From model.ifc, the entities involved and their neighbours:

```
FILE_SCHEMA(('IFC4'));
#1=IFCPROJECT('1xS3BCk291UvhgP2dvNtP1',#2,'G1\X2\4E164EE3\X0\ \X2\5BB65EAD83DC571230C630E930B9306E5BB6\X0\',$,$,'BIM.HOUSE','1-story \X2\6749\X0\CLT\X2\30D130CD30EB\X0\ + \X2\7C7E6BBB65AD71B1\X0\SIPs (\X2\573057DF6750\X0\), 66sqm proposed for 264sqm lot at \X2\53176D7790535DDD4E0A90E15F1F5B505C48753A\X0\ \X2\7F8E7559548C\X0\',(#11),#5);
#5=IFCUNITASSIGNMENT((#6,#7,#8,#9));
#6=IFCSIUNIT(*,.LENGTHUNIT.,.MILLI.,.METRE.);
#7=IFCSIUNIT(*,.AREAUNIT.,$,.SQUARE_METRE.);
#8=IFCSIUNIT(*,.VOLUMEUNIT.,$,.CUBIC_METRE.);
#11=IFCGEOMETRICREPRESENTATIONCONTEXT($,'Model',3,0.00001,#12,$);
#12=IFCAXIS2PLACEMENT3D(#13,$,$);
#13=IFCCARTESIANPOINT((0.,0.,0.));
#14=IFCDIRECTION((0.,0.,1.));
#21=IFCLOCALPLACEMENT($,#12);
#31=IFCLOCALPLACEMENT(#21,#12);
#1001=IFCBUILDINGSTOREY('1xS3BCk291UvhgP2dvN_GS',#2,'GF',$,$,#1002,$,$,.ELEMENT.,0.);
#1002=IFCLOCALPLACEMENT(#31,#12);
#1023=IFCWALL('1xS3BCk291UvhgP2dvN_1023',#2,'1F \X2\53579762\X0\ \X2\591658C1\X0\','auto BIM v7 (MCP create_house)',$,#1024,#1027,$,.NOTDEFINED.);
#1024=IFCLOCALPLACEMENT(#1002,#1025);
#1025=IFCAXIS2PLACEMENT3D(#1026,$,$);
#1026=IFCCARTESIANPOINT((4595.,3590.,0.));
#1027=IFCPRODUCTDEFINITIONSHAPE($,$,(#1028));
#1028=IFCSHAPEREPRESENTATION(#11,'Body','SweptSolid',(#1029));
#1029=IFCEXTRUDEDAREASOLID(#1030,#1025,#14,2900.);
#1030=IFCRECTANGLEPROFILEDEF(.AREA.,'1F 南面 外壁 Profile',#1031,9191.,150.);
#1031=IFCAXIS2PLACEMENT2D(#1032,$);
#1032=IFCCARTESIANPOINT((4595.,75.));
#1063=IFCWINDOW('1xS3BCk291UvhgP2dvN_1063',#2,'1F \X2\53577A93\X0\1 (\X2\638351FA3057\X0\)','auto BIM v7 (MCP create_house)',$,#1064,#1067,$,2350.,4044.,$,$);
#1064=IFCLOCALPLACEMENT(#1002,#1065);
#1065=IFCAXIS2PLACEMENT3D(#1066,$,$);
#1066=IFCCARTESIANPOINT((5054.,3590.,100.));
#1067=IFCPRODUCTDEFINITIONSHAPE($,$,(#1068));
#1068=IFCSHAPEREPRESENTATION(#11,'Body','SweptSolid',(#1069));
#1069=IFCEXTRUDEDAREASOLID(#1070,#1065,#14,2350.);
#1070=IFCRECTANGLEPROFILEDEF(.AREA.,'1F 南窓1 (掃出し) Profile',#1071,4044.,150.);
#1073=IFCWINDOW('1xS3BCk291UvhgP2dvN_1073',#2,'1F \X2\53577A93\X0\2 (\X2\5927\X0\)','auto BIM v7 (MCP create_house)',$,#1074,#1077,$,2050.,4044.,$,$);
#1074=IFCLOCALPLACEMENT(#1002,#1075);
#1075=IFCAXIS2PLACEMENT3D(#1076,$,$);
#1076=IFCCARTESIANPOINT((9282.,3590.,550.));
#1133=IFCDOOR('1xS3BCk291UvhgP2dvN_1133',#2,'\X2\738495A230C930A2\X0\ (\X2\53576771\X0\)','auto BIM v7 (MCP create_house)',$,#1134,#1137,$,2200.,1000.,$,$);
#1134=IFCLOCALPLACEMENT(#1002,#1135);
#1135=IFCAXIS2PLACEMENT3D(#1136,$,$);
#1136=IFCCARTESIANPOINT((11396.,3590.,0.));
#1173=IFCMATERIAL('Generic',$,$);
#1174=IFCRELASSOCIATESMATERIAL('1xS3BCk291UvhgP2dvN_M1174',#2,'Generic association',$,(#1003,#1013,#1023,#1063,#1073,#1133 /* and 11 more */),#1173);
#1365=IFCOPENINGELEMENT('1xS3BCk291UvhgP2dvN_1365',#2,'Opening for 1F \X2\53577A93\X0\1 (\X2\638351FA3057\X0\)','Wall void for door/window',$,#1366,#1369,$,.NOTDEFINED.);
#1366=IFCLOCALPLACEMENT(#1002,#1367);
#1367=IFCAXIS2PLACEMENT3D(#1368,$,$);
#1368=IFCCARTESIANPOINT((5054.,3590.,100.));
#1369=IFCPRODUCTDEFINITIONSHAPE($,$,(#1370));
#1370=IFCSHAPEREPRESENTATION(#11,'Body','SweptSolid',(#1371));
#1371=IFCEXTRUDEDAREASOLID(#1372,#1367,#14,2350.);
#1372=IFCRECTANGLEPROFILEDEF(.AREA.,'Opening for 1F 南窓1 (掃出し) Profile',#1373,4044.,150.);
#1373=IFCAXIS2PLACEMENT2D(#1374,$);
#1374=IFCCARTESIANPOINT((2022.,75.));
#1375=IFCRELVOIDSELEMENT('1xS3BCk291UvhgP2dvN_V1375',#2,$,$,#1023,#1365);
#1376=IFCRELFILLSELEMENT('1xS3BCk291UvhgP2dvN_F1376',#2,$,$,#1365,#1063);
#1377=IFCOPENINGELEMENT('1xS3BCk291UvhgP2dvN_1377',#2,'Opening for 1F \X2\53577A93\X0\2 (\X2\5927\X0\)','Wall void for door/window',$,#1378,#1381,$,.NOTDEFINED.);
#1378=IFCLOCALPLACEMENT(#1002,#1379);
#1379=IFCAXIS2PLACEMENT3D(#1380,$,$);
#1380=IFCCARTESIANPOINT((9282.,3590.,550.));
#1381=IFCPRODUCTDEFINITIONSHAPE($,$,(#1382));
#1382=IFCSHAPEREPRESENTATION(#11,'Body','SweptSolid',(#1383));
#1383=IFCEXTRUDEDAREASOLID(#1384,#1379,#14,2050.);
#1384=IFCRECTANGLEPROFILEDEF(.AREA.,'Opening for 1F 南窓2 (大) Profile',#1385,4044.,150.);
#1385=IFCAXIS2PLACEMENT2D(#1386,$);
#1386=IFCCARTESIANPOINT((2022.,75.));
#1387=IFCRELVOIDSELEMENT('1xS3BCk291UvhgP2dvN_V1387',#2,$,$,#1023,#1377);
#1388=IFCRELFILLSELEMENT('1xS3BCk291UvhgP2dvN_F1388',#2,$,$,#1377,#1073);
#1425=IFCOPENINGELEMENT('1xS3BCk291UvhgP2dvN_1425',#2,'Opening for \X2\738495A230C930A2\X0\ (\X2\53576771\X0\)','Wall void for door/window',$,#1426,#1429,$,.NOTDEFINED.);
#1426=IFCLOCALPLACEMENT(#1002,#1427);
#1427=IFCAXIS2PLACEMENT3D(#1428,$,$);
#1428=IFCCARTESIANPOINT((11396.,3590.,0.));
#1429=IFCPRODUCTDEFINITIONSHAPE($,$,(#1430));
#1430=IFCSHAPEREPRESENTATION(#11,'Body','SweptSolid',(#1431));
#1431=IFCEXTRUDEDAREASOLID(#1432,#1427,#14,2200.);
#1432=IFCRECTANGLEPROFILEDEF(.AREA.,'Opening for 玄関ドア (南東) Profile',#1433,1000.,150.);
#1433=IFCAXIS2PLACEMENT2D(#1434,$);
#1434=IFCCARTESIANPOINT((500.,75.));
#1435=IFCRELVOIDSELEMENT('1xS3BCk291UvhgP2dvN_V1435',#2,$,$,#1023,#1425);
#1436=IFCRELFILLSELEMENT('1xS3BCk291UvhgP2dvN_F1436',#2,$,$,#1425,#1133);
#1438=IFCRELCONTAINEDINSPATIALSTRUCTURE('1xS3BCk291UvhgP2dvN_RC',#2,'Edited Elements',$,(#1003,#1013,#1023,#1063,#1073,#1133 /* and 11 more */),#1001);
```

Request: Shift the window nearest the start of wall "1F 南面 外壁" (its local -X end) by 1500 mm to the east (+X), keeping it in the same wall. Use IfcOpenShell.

```python
import ifcopenshell
import ifcopenshell.api.geometry
import ifcopenshell.util.placement
import ifcopenshell.util.unit

model = ifcopenshell.open("model.ifc")
unit_scale = ifcopenshell.util.unit.calculate_unit_scale(model)

window = model.by_guid("1xS3BCk291UvhgP2dvN_1063")
opening = window.FillsVoids[0].RelatingOpeningElement
wall = opening.VoidsElements[0].RelatingBuildingElement

wall_matrix = ifcopenshell.util.placement.get_local_placement(wall.ObjectPlacement)
shift = wall_matrix[:3, 0] * 1.5 / unit_scale
before = ifcopenshell.util.placement.get_local_placement(window.ObjectPlacement)[:3, 3].copy()

# The window is not placed relative to its opening, so move both.
for product in (opening, window):
    matrix = ifcopenshell.util.placement.get_local_placement(product.ObjectPlacement)
    matrix[:3, 3] += shift
    ifcopenshell.api.geometry.edit_object_placement(model, product=product, matrix=matrix, is_si=False)

after = ifcopenshell.util.placement.get_local_placement(window.ObjectPlacement)[:3, 3]
print("window moved by", (after - before).round(3) + 0.0)

model.write("model_updated.ifc")
```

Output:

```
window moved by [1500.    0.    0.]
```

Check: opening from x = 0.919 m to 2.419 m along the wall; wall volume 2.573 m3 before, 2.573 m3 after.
